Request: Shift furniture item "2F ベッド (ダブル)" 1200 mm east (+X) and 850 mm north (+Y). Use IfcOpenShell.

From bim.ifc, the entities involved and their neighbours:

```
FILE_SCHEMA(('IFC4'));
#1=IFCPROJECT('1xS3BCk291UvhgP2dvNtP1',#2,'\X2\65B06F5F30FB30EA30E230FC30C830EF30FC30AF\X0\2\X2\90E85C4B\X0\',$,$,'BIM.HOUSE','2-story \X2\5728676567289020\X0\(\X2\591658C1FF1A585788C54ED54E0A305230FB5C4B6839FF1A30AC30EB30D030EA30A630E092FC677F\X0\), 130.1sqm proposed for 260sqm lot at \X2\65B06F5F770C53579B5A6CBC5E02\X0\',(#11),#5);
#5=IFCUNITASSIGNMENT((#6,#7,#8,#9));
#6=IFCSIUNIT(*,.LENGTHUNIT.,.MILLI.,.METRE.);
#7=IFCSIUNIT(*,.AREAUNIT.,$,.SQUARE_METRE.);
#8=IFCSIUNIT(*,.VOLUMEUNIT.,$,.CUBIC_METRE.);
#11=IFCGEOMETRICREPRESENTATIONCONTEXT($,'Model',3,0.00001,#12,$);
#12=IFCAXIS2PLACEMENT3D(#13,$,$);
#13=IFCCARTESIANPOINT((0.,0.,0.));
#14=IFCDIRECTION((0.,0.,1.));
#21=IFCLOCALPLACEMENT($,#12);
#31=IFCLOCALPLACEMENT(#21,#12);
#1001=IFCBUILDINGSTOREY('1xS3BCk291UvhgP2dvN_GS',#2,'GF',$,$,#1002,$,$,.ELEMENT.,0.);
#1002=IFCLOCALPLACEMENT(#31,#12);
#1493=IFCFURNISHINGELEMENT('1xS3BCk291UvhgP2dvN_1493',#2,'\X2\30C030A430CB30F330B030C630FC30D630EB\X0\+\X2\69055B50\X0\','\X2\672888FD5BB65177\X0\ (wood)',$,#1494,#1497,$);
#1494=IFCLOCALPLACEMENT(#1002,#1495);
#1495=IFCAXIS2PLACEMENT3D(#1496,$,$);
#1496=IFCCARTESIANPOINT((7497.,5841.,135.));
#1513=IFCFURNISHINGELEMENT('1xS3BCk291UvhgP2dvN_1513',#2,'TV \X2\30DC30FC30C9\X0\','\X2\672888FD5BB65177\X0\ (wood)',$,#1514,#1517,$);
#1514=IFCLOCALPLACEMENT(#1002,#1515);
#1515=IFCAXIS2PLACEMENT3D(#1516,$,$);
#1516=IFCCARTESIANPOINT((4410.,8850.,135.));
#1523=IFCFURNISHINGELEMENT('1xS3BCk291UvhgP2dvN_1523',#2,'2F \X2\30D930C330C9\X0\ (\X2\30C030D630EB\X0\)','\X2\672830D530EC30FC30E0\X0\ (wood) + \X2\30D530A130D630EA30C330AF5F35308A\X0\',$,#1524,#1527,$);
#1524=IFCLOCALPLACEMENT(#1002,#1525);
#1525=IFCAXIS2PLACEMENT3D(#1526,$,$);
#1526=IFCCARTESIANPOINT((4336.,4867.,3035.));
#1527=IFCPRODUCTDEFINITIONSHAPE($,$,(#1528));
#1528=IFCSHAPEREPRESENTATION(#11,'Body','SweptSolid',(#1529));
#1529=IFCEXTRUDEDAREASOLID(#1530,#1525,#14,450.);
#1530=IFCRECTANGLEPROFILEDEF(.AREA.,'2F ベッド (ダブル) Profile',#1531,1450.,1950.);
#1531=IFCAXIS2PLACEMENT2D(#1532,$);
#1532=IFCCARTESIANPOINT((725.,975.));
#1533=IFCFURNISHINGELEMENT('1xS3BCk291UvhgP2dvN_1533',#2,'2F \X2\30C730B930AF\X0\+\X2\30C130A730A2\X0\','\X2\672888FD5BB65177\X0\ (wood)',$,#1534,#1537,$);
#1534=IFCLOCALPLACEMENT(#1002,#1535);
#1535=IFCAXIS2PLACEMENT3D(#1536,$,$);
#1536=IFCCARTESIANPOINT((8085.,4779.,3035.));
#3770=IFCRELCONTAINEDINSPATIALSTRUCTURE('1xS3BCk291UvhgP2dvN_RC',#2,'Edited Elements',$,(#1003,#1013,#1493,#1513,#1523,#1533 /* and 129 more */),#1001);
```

```python
import ifcopenshell
import ifcopenshell.api.geometry
import ifcopenshell.util.placement
import ifcopenshell.util.unit

model = ifcopenshell.open("bim.ifc")
unit_scale = ifcopenshell.util.unit.calculate_unit_scale(model)

item = model.by_guid("1xS3BCk291UvhgP2dvN_1523")
matrix = ifcopenshell.util.placement.get_local_placement(item.ObjectPlacement)
matrix[0, 3] += 1.2 / unit_scale
matrix[1, 3] += 0.85 / unit_scale
ifcopenshell.api.geometry.edit_object_placement(model, product=item, matrix=matrix, is_si=False)

print(ifcopenshell.util.placement.get_local_placement(item.ObjectPlacement).round(3) + 0.0)

model.write("bim-out.ifc")
```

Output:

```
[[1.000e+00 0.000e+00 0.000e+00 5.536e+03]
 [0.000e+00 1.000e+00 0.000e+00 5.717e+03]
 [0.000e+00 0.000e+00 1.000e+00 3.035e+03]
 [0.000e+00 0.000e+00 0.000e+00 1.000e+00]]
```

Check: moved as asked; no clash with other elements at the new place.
